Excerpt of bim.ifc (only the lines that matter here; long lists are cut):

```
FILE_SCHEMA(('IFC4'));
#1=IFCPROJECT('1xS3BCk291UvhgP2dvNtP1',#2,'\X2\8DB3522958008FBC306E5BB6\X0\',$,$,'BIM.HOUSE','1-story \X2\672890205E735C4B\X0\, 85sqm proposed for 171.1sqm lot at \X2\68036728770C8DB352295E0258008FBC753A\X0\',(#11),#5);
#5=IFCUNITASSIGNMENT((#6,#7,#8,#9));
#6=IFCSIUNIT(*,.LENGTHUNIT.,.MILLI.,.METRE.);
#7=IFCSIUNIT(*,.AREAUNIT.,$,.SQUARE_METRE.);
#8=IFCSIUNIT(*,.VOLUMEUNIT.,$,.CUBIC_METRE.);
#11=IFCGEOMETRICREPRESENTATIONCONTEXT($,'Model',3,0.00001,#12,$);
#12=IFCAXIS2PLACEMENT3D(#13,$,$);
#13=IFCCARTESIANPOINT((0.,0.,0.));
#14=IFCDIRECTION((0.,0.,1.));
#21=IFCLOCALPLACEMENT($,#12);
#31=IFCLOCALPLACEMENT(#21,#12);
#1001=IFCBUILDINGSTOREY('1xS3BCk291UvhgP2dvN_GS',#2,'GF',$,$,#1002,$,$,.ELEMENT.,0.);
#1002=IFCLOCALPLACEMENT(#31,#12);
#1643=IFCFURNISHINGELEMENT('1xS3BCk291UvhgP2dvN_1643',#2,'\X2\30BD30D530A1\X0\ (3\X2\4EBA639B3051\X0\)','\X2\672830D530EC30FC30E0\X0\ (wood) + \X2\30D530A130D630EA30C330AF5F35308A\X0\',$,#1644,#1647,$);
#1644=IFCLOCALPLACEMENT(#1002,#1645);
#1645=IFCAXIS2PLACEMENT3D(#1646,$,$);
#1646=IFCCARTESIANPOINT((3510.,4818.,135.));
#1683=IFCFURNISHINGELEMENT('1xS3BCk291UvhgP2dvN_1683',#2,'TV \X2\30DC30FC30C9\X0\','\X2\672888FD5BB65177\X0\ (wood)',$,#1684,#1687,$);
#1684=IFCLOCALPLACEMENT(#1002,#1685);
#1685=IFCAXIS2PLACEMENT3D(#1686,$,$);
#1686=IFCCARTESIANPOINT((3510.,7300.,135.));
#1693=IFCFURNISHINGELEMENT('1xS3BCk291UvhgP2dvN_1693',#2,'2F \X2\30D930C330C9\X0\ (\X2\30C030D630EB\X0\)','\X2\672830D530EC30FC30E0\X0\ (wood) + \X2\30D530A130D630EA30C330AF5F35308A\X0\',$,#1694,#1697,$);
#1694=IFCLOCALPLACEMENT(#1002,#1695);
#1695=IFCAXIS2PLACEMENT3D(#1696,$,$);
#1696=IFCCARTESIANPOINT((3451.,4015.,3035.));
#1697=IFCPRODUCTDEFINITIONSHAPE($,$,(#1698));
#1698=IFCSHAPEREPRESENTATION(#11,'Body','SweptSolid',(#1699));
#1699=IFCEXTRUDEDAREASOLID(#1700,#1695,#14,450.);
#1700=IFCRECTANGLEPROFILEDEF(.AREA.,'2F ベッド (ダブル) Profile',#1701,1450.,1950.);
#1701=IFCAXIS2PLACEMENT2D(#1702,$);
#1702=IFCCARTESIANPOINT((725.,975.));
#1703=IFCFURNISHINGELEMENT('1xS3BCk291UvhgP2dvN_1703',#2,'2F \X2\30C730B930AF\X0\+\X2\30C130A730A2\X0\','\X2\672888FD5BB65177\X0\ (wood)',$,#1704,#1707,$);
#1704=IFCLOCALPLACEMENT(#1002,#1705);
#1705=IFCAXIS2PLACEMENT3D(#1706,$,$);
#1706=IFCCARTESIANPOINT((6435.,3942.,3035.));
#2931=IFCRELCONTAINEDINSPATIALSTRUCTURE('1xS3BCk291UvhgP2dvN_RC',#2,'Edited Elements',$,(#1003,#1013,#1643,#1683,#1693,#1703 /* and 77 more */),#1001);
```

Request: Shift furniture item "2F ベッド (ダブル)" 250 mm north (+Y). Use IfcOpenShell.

```python
import ifcopenshell
import ifcopenshell.api.geometry
import ifcopenshell.util.placement

model = ifcopenshell.open("bim.ifc")

item = model.by_guid("1xS3BCk291UvhgP2dvN_1693")
matrix = ifcopenshell.util.placement.get_local_placement(item.ObjectPlacement)
matrix[1, 3] += 250.0
ifcopenshell.api.geometry.edit_object_placement(model, product=item, matrix=matrix, is_si=False)

print(ifcopenshell.util.placement.get_local_placement(item.ObjectPlacement).round(3) + 0.0)

model.write("bim_v2.ifc")
```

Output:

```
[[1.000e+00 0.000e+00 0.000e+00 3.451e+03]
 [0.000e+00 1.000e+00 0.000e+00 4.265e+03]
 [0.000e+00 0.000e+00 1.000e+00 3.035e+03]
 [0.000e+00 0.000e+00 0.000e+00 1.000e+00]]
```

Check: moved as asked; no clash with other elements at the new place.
